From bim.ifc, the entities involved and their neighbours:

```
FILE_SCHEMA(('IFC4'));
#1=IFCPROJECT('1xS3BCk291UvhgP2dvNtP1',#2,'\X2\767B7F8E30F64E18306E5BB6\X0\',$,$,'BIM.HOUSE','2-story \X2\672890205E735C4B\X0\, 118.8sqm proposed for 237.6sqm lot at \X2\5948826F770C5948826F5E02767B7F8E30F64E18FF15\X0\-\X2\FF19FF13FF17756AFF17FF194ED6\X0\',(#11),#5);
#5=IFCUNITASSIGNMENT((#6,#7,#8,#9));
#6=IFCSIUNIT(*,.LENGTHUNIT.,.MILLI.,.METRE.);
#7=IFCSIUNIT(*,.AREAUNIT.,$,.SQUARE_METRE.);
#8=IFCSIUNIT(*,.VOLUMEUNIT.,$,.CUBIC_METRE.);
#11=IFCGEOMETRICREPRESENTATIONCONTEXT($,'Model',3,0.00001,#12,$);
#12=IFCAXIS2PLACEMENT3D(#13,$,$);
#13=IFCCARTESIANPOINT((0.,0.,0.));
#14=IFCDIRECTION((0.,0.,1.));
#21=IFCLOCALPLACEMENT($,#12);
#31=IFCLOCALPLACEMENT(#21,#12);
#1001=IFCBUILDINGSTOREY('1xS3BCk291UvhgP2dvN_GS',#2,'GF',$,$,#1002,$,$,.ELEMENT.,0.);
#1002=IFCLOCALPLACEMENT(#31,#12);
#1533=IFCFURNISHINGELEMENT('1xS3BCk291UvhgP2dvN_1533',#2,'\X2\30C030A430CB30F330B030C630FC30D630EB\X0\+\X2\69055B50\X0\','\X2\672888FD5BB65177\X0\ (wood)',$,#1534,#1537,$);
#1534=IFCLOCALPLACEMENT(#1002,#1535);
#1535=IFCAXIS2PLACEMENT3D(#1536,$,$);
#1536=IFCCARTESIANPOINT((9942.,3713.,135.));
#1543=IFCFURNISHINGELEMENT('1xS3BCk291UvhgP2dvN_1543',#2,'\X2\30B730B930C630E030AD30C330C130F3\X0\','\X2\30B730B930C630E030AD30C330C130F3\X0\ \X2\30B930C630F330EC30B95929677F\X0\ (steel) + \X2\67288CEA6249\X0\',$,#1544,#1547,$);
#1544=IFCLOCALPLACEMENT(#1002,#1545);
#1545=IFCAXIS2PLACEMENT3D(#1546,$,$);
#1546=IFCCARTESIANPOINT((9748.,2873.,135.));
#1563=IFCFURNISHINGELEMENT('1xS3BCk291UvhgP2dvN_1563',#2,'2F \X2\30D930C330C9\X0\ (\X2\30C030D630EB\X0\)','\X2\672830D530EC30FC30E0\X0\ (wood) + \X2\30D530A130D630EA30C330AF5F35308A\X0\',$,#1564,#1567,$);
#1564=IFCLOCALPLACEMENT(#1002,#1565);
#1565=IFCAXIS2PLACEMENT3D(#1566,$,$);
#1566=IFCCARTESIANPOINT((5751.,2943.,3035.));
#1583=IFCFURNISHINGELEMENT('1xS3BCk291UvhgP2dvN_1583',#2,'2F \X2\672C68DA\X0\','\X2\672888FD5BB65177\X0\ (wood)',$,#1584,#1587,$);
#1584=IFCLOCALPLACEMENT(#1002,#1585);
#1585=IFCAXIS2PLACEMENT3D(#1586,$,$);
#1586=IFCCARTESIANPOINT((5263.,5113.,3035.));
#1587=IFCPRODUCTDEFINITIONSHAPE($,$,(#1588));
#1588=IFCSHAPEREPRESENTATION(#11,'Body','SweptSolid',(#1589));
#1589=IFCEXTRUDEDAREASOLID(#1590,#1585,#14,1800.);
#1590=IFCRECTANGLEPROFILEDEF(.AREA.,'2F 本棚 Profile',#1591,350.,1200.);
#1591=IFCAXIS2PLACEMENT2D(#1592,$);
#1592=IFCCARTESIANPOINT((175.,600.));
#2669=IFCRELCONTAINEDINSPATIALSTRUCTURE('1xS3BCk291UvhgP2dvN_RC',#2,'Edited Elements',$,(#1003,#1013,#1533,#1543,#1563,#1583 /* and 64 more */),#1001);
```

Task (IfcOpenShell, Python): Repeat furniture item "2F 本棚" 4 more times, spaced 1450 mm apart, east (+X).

```python
import numpy as np
import ifcopenshell
import ifcopenshell.api.geometry
import ifcopenshell.api.root
import ifcopenshell.util.element
import ifcopenshell.util.placement

model = ifcopenshell.open("bim.ifc")


def reuse_history(source, copy):
    """copy_class also copies each property set's owner history, people and application; keep the originals."""
    for rel in copy.IsDefinedBy:
        if rel.is_a("IfcRelDefinesByProperties") and (history := rel.RelatingPropertyDefinition.OwnerHistory):
            rel.RelatingPropertyDefinition.OwnerHistory = source.OwnerHistory
            ifcopenshell.util.element.remove_deep2(model, history)


source = model.by_guid("1xS3BCk291UvhgP2dvN_1583")
base = ifcopenshell.util.placement.get_local_placement(source.ObjectPlacement)
step = np.array([1.0, 0.0, 0.0]) * 1450.0

for i in range(1, 5):
    copy = ifcopenshell.api.root.copy_class(model, product=source)
    copy.Representation = ifcopenshell.util.element.copy_deep(
        model, source.Representation, exclude=["IfcGeometricRepresentationContext", "IfcRepresentationMap"]
    )
    reuse_history(source, copy)
    matrix = base.copy()
    matrix[:3, 3] += i * step
    print("added at", matrix[:3, 3].round(3) + 0.0)
    ifcopenshell.api.geometry.edit_object_placement(model, product=copy, matrix=matrix, is_si=False)

model.write("bim_v2.ifc")
```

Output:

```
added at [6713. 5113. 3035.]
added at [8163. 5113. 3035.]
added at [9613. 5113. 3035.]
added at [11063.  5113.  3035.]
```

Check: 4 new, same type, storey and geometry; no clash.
